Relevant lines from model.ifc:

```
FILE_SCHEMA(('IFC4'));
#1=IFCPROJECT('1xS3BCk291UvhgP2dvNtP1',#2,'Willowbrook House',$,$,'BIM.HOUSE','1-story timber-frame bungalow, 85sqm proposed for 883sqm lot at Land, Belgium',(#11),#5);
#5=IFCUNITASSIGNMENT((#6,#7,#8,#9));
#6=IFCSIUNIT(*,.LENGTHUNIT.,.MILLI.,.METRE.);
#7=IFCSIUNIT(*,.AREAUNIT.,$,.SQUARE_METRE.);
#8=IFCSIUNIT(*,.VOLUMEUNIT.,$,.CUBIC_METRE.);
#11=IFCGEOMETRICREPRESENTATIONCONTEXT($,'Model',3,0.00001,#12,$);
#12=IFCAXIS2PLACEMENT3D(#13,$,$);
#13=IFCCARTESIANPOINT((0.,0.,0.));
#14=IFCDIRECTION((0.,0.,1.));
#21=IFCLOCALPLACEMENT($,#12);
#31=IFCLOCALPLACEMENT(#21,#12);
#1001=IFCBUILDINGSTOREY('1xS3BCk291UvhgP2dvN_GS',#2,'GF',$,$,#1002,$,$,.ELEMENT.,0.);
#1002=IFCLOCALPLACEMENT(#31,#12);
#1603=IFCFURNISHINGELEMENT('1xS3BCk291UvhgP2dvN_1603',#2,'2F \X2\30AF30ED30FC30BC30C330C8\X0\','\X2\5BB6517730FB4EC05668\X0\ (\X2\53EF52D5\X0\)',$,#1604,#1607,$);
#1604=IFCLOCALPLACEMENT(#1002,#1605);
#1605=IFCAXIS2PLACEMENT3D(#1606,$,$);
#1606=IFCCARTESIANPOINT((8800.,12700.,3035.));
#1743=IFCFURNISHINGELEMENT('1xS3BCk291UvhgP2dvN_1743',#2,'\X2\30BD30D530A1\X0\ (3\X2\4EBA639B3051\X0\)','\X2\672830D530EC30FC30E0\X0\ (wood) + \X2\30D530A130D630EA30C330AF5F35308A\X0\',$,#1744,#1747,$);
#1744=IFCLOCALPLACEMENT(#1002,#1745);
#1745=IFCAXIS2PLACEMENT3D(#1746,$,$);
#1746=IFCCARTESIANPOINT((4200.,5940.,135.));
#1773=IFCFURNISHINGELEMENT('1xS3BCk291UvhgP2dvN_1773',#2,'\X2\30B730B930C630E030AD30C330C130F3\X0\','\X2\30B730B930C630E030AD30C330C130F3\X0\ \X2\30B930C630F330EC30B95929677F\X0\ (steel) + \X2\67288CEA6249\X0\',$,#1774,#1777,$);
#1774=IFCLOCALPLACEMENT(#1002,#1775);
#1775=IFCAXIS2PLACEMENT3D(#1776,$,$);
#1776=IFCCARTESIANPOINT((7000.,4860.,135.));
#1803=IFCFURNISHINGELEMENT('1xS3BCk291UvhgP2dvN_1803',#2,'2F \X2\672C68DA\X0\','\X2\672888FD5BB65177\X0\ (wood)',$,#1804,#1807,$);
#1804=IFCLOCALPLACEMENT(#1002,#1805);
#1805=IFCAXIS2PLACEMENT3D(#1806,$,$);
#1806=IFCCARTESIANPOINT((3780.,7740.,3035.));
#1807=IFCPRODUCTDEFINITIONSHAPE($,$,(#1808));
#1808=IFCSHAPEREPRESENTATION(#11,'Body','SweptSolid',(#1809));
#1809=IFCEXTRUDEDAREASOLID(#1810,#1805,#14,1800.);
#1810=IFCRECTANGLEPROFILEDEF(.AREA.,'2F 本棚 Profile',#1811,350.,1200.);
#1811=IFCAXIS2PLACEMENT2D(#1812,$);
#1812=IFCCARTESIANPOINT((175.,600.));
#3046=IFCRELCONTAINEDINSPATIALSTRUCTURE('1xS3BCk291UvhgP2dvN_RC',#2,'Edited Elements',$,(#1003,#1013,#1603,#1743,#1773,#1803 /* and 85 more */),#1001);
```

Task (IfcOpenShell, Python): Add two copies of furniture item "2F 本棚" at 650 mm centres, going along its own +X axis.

```python
import ifcopenshell
import ifcopenshell.api.geometry
import ifcopenshell.api.root
import ifcopenshell.util.element
import ifcopenshell.util.placement
import ifcopenshell.util.unit

model = ifcopenshell.open("model.ifc")
unit_scale = ifcopenshell.util.unit.calculate_unit_scale(model)


def reuse_history(source, copy):
    """copy_class also copies each property set's owner history, people and application; keep the originals."""
    for rel in copy.IsDefinedBy:
        if rel.is_a("IfcRelDefinesByProperties") and (history := rel.RelatingPropertyDefinition.OwnerHistory):
            rel.RelatingPropertyDefinition.OwnerHistory = source.OwnerHistory
            ifcopenshell.util.element.remove_deep2(model, history)


source = model.by_id(1803)
base = ifcopenshell.util.placement.get_local_placement(source.ObjectPlacement)
step = base[:3, 0] * 0.65 / unit_scale

for i in range(1, 3):
    copy = ifcopenshell.api.root.copy_class(model, product=source)
    copy.Representation = ifcopenshell.util.element.copy_deep(
        model, source.Representation, exclude=["IfcGeometricRepresentationContext", "IfcRepresentationMap"]
    )
    reuse_history(source, copy)
    matrix = base.copy()
    matrix[:3, 3] += i * step
    print("added at", matrix[:3, 3].round(3) + 0.0)
    ifcopenshell.api.geometry.edit_object_placement(model, product=copy, matrix=matrix, is_si=False)

model.write("model_updated.ifc")
```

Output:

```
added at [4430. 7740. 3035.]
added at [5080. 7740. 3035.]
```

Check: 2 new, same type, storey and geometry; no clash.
